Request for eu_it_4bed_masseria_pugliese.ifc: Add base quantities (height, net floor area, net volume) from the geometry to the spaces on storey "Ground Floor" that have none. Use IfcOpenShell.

First a look at what the model holds.

```python
import ifcopenshell
import ifcopenshell.util.element
import ifcopenshell.util.unit

model = ifcopenshell.open("eu_it_4bed_masseria_pugliese.ifc")
print(model.schema)
for unit_type in ("LENGTHUNIT", "AREAUNIT", "VOLUMEUNIT"):
    print(unit_type, ifcopenshell.util.unit.calculate_unit_scale(model, unit_type))
storey = next(s for s in model.by_type("IfcBuildingStorey") if s.Name == "Ground Floor")
spaces = [e for e in ifcopenshell.util.element.get_decomposition(storey) if e.is_a("IfcSpace")]
for e in sorted(spaces, key=lambda e: e.id()):
    print(e.id(), e.is_a(), e.Name, list(ifcopenshell.util.element.get_psets(e, qtos_only=True)), sep=" | ")
```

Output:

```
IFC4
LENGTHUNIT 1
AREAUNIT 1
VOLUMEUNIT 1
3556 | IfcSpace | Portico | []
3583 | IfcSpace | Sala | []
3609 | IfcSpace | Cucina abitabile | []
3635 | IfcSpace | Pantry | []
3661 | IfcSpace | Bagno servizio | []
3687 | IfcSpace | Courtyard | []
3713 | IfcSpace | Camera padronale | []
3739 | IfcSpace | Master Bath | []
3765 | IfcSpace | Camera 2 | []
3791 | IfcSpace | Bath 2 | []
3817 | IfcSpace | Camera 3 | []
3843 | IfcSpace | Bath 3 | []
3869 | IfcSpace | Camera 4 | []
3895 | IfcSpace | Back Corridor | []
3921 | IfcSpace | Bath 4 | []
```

```python
import ifcopenshell
import ifcopenshell.api.pset
import ifcopenshell.geom
import ifcopenshell.util.element
import ifcopenshell.util.shape
import ifcopenshell.util.unit

model = ifcopenshell.open("eu_it_4bed_masseria_pugliese.ifc")
unit_scale = ifcopenshell.util.unit.calculate_unit_scale(model)
area_scale = ifcopenshell.util.unit.calculate_unit_scale(model, "AREAUNIT")
volume_scale = ifcopenshell.util.unit.calculate_unit_scale(model, "VOLUMEUNIT")
settings = ifcopenshell.geom.settings()

storey = next(s for s in model.by_type("IfcBuildingStorey") if s.Name == "Ground Floor")
spaces = [e for e in ifcopenshell.util.element.get_decomposition(storey) if e.is_a("IfcSpace")]

for e in sorted(spaces, key=lambda e: e.id()):
    if ifcopenshell.util.element.get_psets(e, qtos_only=True, should_inherit=False):
        continue
    # Geometry comes back in metres, in the element's own axes.
    shape = ifcopenshell.geom.create_shape(settings, e)
    values = {
        "Height": ifcopenshell.util.shape.get_z(shape.geometry) / unit_scale,
        "NetFloorArea": ifcopenshell.util.shape.get_footprint_area(shape.geometry) / area_scale,
        "NetVolume": ifcopenshell.util.shape.get_volume(shape.geometry) / volume_scale,
    }
    qto = ifcopenshell.api.pset.add_qto(model, product=e, name="Qto_SpaceBaseQuantities")
    ifcopenshell.api.pset.edit_qto(model, qto=qto, properties=values)
    print(e.id(), {k: round(v, 3) for k, v in values.items()})

model.write("eu_it_4bed_masseria_pugliese_rev.ifc")
```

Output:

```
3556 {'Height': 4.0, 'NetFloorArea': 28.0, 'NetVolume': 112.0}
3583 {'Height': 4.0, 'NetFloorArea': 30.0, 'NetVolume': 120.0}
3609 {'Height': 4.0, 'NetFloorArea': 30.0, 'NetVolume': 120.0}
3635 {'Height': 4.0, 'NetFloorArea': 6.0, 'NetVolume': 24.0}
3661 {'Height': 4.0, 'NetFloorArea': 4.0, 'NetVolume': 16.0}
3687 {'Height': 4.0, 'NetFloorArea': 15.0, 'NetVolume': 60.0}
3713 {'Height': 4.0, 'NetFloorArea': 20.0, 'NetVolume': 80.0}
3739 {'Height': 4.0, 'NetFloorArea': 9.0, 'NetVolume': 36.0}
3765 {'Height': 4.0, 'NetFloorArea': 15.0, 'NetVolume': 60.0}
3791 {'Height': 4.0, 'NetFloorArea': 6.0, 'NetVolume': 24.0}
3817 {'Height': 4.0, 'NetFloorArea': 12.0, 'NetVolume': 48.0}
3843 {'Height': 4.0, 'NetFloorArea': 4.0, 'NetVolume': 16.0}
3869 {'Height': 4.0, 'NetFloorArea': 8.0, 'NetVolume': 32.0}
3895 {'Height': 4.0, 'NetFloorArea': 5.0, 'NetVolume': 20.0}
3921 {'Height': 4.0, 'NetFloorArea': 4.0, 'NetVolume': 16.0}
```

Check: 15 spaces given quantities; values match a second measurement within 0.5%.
